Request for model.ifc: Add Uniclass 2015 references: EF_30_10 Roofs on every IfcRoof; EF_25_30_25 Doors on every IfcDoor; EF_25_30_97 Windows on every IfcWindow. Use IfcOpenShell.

First a look at what the model holds.

```python
import ifcopenshell

model = ifcopenshell.open("model.ifc")
print(model.schema)
print("classifications:", [c.Name for c in model.by_type("IfcClassification")])
for ifc_class in ("IfcDoor", "IfcRoof", "IfcStair", "IfcWall", "IfcWindow"):
    print(ifc_class, len(model.by_type(ifc_class)))
```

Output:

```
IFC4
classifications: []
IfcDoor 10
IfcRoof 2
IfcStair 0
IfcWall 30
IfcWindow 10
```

```python
import ifcopenshell
import ifcopenshell.api.classification

model = ifcopenshell.open("model.ifc")

system = ifcopenshell.api.classification.add_classification(model, classification="Uniclass 2015")

codes = {
    "IfcRoof": ("EF_30_10", "Roofs"),
    "IfcDoor": ("EF_25_30_25", "Doors"),
    "IfcWindow": ("EF_25_30_97", "Windows"),
}
for ifc_class, (code, name) in codes.items():
    products = model.by_type(ifc_class)
    ifcopenshell.api.classification.add_reference(
        model, products=products, classification=system, identification=code, name=name
    )
    print(code, len(products))

model.write("model_updated.ifc")
```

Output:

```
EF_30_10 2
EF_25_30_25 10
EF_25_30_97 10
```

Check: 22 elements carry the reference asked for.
